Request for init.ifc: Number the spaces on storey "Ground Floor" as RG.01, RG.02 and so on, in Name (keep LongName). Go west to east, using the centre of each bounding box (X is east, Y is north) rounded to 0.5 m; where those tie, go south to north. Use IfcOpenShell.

First a look at what the model holds.

```python
import ifcopenshell
import ifcopenshell.util.element
import ifcopenshell.util.placement

model = ifcopenshell.open("init.ifc")
print(model.schema)
storey = next(s for s in model.by_type("IfcBuildingStorey") if s.Name == "Ground Floor")
spaces = [e for e in ifcopenshell.util.element.get_decomposition(storey) if e.is_a("IfcSpace")]
for e in sorted(spaces, key=lambda e: e.id()):
    origin = ifcopenshell.util.placement.get_local_placement(e.ObjectPlacement)[:3, 3]
    print(e.id(), e.Name, e.LongName, origin.round(2) + 0.0, sep=" | ")
```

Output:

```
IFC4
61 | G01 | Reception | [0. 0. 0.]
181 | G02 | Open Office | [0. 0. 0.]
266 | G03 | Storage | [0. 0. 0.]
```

```python
import ifcopenshell
import ifcopenshell.geom
import ifcopenshell.util.element
import ifcopenshell.util.shape

model = ifcopenshell.open("init.ifc")
settings = ifcopenshell.geom.settings()
settings.set("use-world-coords", True)


def centre(element):
    shape = ifcopenshell.geom.create_shape(settings, element)
    return ifcopenshell.util.shape.get_bbox_centroid(shape.geometry)


storey = next(s for s in model.by_type("IfcBuildingStorey") if s.Name == "Ground Floor")
spaces = [e for e in ifcopenshell.util.element.get_decomposition(storey) if e.is_a("IfcSpace")]

# Insertion points can sit at a corner or the storey origin, so sort by the geometry (in metres).
centres = {e: centre(e) for e in spaces}
spaces.sort(key=lambda e: (round(centres[e][0] / 0.5), centres[e][1]))

for i, e in enumerate(spaces, start=1):
    number = f"RG.{i:02d}"
    e.Name = number
    print(e.id(), number)

model.write("init_rev.ifc")
```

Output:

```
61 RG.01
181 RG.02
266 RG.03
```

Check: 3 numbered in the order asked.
